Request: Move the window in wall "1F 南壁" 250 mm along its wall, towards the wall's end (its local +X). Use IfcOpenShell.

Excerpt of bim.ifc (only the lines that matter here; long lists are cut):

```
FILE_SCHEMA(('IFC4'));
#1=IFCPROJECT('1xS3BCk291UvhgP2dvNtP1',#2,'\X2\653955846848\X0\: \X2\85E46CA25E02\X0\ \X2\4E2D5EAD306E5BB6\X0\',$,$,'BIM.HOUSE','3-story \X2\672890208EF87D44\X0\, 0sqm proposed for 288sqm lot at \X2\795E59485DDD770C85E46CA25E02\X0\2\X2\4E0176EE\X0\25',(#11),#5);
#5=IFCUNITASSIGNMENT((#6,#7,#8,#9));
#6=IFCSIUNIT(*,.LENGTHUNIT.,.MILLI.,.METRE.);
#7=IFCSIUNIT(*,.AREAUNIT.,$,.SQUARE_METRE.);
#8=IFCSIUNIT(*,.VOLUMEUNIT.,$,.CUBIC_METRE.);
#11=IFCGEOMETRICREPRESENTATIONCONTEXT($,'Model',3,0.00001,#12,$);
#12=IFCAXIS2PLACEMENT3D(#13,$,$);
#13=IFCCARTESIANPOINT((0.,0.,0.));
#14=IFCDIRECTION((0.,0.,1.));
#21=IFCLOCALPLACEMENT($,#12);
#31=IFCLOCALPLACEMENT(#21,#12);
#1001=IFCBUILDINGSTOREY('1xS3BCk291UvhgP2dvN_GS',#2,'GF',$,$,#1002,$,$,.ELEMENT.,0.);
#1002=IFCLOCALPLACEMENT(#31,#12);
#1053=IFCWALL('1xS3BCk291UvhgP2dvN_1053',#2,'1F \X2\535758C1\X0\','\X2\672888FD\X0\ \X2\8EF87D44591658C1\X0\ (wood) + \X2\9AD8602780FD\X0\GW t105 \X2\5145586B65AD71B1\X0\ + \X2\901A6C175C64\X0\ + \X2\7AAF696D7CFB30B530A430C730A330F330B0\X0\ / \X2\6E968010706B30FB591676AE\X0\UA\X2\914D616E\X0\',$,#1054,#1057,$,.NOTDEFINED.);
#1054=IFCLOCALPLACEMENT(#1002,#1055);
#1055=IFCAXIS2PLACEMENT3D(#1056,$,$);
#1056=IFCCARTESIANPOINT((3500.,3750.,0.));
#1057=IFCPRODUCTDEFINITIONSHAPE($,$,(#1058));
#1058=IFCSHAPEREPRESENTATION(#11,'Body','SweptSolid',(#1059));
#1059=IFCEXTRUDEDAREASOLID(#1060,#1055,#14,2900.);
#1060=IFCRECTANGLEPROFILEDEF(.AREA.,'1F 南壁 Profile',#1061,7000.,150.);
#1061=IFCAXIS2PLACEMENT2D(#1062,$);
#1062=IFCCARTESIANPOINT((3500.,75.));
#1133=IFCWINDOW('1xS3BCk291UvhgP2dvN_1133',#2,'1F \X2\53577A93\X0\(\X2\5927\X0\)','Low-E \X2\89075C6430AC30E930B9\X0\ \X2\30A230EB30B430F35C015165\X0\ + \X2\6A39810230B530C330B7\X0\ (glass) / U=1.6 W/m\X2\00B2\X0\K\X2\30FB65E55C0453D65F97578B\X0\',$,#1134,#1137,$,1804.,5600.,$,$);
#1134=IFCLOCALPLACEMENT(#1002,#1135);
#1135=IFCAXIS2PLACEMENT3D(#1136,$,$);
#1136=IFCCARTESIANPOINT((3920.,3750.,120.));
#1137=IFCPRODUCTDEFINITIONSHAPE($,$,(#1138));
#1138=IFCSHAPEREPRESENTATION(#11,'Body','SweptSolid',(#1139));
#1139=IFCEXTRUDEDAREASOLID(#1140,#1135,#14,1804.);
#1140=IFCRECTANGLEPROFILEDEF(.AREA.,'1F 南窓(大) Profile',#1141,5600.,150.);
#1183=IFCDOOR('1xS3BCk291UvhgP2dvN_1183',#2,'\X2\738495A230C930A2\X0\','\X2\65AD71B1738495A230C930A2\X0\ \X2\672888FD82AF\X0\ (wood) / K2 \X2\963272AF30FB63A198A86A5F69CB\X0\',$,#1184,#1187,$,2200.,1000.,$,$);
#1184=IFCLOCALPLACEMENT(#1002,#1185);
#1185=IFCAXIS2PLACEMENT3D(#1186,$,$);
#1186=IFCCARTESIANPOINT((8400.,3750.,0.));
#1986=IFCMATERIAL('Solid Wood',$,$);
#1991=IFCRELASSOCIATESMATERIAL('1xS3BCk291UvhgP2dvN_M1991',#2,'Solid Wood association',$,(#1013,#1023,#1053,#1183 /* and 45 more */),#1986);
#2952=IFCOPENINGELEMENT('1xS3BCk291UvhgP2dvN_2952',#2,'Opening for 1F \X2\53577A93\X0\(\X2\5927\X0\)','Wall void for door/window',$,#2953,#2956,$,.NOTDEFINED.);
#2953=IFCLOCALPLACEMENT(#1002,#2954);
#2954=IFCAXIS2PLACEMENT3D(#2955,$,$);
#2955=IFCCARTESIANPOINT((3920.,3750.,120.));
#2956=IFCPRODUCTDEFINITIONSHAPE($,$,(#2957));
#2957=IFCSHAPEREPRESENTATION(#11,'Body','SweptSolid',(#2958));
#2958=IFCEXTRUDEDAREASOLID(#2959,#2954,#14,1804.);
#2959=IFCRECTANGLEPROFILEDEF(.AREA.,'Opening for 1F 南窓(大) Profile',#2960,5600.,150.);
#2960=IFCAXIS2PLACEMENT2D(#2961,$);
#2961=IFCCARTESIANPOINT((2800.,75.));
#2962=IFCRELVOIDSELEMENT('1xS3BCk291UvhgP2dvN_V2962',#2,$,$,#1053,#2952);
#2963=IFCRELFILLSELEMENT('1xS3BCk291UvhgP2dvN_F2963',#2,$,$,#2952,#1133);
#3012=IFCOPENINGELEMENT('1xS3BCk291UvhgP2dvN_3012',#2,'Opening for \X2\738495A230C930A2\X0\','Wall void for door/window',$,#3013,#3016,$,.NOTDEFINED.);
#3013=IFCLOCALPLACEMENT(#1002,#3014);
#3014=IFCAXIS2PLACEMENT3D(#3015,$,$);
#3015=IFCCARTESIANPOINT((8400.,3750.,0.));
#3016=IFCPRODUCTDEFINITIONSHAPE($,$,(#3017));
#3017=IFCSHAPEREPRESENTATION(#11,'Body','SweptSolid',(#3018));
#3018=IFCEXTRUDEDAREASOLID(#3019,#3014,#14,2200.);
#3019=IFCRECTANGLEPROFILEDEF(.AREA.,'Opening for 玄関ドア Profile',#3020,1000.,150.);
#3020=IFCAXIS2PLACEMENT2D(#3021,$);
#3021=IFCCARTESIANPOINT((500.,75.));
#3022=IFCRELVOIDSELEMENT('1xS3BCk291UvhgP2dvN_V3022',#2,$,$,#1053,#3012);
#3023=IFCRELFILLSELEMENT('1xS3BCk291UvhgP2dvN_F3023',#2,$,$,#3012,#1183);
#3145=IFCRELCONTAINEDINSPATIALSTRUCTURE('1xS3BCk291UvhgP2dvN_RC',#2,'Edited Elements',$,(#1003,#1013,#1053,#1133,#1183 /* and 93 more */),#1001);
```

```python
import ifcopenshell
import ifcopenshell.api.geometry
import ifcopenshell.util.placement
import ifcopenshell.util.unit

model = ifcopenshell.open("bim.ifc")
unit_scale = ifcopenshell.util.unit.calculate_unit_scale(model)

window = model.by_guid("1xS3BCk291UvhgP2dvN_1133")
opening = window.FillsVoids[0].RelatingOpeningElement
wall = opening.VoidsElements[0].RelatingBuildingElement

wall_matrix = ifcopenshell.util.placement.get_local_placement(wall.ObjectPlacement)
shift = wall_matrix[:3, 0] * 0.25 / unit_scale
before = ifcopenshell.util.placement.get_local_placement(window.ObjectPlacement)[:3, 3].copy()

# The window is not placed relative to its opening, so move both.
for product in (opening, window):
    matrix = ifcopenshell.util.placement.get_local_placement(product.ObjectPlacement)
    matrix[:3, 3] += shift
    ifcopenshell.api.geometry.edit_object_placement(model, product=product, matrix=matrix, is_si=False)

after = ifcopenshell.util.placement.get_local_placement(window.ObjectPlacement)[:3, 3]
print("window moved by", (after - before).round(3) + 0.0)

model.write("bim-out.ifc")
```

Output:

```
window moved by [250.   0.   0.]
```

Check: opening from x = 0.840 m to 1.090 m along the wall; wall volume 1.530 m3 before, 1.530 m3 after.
